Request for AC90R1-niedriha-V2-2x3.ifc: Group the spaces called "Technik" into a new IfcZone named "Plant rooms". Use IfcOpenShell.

First a look at what the model holds.

```python
import ifcopenshell

model = ifcopenshell.open("AC90R1-niedriha-V2-2x3.ifc")
print(model.schema)
seen = {}
for space in model.by_type("IfcSpace"):
    seen[space.LongName] = seen.get(space.LongName, 0) + 1
for name, count in sorted(seen.items(), key=str):
    print(count, "x", name)
print("zones:", [z.Name for z in model.by_type("IfcZone")][:20])
```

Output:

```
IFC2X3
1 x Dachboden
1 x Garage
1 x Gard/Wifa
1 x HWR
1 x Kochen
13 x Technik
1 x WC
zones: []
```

```python
import ifcopenshell
import ifcopenshell.api.group
import ifcopenshell.api.root

model = ifcopenshell.open("AC90R1-niedriha-V2-2x3.ifc")

names = {"Technik"}
spaces = [s for s in model.by_type("IfcSpace") if s.LongName in names]

zone = ifcopenshell.api.root.create_entity(model, ifc_class="IfcZone", name="Plant rooms")
ifcopenshell.api.group.assign_group(model, products=spaces, group=zone)
print(len(spaces), "spaces in", zone.Name)

model.write("AC90R1-niedriha-V2-2x3_v2.ifc")
```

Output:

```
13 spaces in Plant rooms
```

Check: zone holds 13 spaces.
